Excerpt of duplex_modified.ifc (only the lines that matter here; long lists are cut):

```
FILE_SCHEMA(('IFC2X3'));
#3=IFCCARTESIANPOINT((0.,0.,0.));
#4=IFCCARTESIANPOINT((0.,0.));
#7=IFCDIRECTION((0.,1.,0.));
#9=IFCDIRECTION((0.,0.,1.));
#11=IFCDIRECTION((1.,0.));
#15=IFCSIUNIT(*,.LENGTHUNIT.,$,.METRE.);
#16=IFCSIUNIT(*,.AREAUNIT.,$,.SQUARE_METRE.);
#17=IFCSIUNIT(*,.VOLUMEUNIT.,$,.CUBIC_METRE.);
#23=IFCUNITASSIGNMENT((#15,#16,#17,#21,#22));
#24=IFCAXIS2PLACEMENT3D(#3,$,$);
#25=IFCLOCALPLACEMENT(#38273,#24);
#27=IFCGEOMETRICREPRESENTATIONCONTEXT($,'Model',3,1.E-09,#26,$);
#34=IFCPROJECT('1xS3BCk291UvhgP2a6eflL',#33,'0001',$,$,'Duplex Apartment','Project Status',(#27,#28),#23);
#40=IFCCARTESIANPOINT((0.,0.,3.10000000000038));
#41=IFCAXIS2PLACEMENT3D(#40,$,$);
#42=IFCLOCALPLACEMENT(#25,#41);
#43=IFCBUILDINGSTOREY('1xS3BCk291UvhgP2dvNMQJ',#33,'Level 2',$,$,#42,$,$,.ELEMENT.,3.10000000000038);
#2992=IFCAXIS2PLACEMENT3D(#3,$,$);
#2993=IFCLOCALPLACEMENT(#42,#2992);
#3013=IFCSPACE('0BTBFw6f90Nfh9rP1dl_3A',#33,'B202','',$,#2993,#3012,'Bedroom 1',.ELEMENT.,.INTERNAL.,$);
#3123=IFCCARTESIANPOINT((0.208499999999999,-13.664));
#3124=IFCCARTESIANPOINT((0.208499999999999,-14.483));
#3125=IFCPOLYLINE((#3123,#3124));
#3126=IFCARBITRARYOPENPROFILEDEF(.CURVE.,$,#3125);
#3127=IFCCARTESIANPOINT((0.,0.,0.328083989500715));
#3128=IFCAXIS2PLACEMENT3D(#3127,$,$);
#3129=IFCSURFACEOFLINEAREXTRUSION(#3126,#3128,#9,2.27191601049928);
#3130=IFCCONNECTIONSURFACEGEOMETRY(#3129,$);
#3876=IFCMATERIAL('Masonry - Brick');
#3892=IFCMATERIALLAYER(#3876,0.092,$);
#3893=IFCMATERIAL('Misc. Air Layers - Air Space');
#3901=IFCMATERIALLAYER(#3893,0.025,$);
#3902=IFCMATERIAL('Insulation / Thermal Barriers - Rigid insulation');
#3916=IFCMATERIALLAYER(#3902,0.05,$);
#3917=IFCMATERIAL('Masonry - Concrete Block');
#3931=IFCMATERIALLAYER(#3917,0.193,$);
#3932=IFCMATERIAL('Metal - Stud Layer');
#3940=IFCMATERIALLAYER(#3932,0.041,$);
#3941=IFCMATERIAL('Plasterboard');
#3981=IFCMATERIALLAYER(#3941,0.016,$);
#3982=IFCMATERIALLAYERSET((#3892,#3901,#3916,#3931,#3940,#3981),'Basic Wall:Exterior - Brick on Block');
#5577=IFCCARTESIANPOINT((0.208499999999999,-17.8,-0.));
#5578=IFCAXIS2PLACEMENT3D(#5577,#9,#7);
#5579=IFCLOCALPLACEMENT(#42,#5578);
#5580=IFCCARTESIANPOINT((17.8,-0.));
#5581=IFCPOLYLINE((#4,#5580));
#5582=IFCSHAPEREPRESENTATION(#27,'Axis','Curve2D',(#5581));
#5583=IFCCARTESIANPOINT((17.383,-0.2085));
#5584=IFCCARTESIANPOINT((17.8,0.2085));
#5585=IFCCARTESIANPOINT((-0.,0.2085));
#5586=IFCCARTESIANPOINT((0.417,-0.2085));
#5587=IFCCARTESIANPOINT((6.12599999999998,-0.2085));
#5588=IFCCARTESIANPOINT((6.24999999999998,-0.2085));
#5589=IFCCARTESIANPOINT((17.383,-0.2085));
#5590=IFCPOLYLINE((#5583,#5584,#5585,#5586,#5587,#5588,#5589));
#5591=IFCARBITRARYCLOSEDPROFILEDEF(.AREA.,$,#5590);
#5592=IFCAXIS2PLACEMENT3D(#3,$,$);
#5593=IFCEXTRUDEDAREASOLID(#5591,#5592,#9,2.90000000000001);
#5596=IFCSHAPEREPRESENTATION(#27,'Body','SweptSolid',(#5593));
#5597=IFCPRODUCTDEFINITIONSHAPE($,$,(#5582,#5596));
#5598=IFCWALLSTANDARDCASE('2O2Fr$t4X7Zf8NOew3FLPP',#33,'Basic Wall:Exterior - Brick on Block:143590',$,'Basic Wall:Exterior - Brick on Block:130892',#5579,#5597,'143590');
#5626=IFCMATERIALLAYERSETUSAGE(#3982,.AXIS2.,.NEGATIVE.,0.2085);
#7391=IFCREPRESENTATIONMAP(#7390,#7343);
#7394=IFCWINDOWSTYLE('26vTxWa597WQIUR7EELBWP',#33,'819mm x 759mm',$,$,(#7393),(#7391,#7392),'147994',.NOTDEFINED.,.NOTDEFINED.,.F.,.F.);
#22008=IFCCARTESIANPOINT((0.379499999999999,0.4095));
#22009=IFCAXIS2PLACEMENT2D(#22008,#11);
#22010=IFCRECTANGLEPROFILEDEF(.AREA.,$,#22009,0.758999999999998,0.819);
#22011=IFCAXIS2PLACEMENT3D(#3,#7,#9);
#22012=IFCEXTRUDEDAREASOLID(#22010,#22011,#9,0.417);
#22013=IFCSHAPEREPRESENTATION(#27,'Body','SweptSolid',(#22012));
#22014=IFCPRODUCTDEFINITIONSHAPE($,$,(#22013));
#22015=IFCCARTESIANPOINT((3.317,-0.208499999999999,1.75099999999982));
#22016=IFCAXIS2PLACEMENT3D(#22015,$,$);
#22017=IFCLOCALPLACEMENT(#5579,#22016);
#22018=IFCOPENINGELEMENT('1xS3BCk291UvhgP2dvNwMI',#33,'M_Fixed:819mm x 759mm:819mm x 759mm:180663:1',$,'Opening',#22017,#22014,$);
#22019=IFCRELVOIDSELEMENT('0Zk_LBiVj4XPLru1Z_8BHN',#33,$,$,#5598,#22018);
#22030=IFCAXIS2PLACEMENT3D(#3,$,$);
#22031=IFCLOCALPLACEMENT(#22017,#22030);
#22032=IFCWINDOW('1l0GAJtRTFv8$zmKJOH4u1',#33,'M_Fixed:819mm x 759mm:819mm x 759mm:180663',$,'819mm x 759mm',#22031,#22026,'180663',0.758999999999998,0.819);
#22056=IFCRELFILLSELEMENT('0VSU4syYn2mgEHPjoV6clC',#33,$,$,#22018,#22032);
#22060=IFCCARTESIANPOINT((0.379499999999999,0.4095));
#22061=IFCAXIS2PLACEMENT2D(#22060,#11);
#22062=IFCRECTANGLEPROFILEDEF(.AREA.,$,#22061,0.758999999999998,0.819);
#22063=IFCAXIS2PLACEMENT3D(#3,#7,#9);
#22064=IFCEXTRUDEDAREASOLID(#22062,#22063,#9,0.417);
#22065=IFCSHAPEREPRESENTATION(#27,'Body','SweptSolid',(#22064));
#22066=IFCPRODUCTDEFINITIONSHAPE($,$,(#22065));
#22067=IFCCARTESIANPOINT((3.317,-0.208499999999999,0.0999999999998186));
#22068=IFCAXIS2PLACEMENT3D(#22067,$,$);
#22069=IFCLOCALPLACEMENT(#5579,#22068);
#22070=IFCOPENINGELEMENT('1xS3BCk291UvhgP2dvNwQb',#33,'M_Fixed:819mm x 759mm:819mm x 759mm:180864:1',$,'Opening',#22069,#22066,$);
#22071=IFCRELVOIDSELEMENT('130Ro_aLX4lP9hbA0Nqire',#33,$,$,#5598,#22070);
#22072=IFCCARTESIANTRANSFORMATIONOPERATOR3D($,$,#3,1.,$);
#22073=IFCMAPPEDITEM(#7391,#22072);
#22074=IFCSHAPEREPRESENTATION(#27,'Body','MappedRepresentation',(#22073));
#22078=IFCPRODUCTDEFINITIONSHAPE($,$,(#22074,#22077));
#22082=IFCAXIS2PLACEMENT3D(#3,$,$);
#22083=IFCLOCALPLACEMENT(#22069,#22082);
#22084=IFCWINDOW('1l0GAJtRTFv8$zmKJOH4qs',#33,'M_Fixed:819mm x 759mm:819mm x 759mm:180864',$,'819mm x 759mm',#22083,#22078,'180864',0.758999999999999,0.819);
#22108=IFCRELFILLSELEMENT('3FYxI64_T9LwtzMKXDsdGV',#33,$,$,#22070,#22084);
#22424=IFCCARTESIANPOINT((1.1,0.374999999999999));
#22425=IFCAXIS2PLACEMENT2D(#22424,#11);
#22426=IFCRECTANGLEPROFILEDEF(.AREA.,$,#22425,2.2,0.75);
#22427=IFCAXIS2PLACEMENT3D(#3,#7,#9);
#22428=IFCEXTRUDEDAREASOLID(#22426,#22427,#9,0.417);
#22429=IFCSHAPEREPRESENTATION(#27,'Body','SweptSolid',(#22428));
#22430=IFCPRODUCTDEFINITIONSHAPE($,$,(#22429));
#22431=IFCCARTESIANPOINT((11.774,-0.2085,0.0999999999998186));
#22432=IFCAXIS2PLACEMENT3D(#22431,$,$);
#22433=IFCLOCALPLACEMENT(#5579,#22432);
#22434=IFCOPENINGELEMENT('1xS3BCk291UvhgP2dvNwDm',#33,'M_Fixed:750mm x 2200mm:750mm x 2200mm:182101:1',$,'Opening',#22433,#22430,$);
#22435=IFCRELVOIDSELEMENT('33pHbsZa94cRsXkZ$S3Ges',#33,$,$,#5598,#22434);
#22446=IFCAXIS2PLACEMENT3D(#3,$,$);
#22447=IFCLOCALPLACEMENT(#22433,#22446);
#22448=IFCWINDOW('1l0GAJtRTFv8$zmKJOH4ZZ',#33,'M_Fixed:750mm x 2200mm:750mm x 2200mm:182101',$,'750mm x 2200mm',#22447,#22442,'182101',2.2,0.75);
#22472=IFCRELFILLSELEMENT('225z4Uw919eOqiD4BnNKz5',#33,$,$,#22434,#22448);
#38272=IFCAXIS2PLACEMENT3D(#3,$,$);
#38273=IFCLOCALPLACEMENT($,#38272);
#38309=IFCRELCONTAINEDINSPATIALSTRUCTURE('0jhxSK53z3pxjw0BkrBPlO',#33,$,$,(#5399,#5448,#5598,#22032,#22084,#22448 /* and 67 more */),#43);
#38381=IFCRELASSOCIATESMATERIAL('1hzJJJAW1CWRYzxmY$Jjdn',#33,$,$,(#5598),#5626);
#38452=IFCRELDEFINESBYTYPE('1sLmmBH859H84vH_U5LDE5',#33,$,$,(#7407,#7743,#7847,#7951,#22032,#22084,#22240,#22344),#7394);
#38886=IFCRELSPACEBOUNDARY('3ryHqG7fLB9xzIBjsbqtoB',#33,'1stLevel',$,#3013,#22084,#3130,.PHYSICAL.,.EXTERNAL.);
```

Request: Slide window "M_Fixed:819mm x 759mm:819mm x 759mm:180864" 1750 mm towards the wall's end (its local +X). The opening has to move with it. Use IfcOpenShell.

```python
import numpy as np
import ifcopenshell
import ifcopenshell.api.geometry
import ifcopenshell.util.placement

model = ifcopenshell.open("duplex_modified.ifc")

window = model.by_guid("1l0GAJtRTFv8$zmKJOH4qs")
opening = window.FillsVoids[0].RelatingOpeningElement
wall = opening.VoidsElements[0].RelatingBuildingElement

wall_matrix = ifcopenshell.util.placement.get_local_placement(wall.ObjectPlacement)
shift = wall_matrix[:3, 0] * 1.75
before = ifcopenshell.util.placement.get_local_placement(window.ObjectPlacement)[:3, 3].copy()

# The window is placed relative to its opening, so it follows when the opening moves.
matrix = ifcopenshell.util.placement.get_local_placement(opening.ObjectPlacement)
matrix[:3, 3] += shift
ifcopenshell.api.geometry.edit_object_placement(
    model, product=opening, matrix=matrix, is_si=False, should_transform_children=True
)

# Space boundary surfaces are stored in each space's coordinates; move them too.
for rel in window.ProvidesBoundaries:
    if not rel.ConnectionGeometry:
        continue
    surface = rel.ConnectionGeometry.SurfaceOnRelatingElement
    space_matrix = ifcopenshell.util.placement.get_local_placement(rel.RelatingSpace.ObjectPlacement)
    point = np.array(surface.Position.Location.Coordinates) + space_matrix[:3, :3].T @ shift
    surface.Position = model.createIfcAxis2Placement3D(
        model.createIfcCartesianPoint(point.tolist()), surface.Position.Axis, surface.Position.RefDirection
    )

after = ifcopenshell.util.placement.get_local_placement(window.ObjectPlacement)[:3, 3]
print("window moved by", (after - before).round(3) + 0.0)

model.write("duplex_modified-out.ifc")
```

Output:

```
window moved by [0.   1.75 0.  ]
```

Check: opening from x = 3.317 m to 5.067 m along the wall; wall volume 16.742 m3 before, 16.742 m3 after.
